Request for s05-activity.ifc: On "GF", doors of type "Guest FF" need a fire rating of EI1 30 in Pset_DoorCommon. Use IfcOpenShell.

First a look at what the model holds.

```python
import ifcopenshell
import ifcopenshell.util.element

model = ifcopenshell.open("s05-activity.ifc")
print(model.schema)
storey = next(s for s in model.by_type("IfcBuildingStorey") if s.Name == "GF")
doors = [e for e in ifcopenshell.util.element.get_decomposition(storey) if e.is_a("IfcDoor")]
seen = {}
for e in doors:
    element_type = ifcopenshell.util.element.get_type(e)
    key = (element_type.Name if element_type != e and element_type else None, ifcopenshell.util.element.get_pset(e, "Pset_DoorCommon", "FireRating"))
    seen[key] = seen.get(key, 0) + 1
for (name, value), count in sorted(seen.items(), key=str):
    print(count, "x", name, "|", value)
```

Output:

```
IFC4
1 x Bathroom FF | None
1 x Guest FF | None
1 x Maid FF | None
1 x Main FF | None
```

```python
import ifcopenshell
import ifcopenshell.api.pset
import ifcopenshell.util.element

model = ifcopenshell.open("s05-activity.ifc")

storey = next(s for s in model.by_type("IfcBuildingStorey") if s.Name == "GF")
doors = [e for e in ifcopenshell.util.element.get_decomposition(storey) if e.is_a("IfcDoor")]

count = 0
for e in doors:
    element_type = ifcopenshell.util.element.get_type(e)
    if element_type in (None, e) or element_type.Name != "Guest FF":
        continue
    # add_pset returns the element's existing set when there is one.
    pset = ifcopenshell.api.pset.add_pset(model, product=e, name="Pset_DoorCommon")
    ifcopenshell.api.pset.edit_pset(model, pset=pset, properties={"FireRating": "EI1 30"})
    count += 1

print(count, "doors updated")

model.write("s05-activity_v2.ifc")
```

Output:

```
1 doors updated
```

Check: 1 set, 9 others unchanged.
